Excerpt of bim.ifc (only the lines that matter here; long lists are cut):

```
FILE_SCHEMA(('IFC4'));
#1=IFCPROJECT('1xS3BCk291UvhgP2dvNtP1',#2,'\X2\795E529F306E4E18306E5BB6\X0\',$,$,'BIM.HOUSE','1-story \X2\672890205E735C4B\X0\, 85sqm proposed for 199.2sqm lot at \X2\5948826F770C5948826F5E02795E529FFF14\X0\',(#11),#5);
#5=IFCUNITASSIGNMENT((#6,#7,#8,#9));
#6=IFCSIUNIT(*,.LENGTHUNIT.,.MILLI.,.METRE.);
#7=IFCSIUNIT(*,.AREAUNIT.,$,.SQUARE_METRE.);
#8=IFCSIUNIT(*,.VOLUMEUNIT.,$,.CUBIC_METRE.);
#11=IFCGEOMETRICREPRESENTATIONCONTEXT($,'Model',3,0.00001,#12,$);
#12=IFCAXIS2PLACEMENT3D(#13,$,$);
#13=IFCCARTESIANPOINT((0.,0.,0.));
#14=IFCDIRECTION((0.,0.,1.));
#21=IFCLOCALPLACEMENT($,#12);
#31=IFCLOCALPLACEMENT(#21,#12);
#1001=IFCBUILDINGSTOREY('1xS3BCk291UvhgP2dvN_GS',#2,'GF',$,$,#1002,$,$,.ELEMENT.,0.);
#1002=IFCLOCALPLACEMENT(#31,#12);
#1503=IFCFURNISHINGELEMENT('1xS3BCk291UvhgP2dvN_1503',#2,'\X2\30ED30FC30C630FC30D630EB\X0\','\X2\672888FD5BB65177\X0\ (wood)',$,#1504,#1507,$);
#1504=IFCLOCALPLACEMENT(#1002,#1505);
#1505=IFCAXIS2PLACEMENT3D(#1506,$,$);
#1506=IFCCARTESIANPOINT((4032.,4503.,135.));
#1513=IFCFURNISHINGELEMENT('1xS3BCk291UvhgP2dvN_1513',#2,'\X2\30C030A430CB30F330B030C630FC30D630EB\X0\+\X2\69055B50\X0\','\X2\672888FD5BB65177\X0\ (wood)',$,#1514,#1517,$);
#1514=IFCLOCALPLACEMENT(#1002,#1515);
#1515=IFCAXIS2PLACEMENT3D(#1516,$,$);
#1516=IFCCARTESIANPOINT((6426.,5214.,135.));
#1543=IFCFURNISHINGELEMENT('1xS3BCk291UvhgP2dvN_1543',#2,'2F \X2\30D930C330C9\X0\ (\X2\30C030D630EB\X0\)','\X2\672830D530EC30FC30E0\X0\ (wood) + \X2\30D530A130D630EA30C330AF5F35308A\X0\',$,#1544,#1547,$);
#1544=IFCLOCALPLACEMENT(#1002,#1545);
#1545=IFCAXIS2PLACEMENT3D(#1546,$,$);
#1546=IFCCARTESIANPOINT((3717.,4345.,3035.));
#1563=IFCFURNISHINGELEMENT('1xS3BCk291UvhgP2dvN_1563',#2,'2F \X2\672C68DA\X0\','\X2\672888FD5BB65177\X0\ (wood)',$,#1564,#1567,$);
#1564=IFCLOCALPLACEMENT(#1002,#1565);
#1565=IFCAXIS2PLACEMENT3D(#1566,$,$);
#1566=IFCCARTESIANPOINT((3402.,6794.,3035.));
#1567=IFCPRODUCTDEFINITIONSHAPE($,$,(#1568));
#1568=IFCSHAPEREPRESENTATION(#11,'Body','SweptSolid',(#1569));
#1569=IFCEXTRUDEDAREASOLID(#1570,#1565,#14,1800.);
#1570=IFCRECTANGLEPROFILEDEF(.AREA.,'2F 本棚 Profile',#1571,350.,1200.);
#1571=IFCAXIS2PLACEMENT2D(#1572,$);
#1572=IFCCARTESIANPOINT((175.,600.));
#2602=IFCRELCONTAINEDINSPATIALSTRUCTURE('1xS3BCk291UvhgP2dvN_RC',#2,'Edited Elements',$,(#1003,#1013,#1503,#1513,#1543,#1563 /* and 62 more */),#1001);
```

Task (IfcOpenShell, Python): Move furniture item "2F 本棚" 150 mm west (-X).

```python
import ifcopenshell
import ifcopenshell.api.geometry
import ifcopenshell.util.placement
import ifcopenshell.util.unit

model = ifcopenshell.open("bim.ifc")
unit_scale = ifcopenshell.util.unit.calculate_unit_scale(model)

item = model.by_id(1563)
matrix = ifcopenshell.util.placement.get_local_placement(item.ObjectPlacement)
matrix[0, 3] -= 0.15 / unit_scale
ifcopenshell.api.geometry.edit_object_placement(model, product=item, matrix=matrix, is_si=False)

print(ifcopenshell.util.placement.get_local_placement(item.ObjectPlacement).round(3) + 0.0)

model.write("bim_rev.ifc")
```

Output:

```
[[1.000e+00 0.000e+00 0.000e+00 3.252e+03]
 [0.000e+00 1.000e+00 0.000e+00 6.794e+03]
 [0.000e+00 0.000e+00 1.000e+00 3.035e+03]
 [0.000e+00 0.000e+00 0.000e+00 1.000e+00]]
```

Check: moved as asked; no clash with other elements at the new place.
